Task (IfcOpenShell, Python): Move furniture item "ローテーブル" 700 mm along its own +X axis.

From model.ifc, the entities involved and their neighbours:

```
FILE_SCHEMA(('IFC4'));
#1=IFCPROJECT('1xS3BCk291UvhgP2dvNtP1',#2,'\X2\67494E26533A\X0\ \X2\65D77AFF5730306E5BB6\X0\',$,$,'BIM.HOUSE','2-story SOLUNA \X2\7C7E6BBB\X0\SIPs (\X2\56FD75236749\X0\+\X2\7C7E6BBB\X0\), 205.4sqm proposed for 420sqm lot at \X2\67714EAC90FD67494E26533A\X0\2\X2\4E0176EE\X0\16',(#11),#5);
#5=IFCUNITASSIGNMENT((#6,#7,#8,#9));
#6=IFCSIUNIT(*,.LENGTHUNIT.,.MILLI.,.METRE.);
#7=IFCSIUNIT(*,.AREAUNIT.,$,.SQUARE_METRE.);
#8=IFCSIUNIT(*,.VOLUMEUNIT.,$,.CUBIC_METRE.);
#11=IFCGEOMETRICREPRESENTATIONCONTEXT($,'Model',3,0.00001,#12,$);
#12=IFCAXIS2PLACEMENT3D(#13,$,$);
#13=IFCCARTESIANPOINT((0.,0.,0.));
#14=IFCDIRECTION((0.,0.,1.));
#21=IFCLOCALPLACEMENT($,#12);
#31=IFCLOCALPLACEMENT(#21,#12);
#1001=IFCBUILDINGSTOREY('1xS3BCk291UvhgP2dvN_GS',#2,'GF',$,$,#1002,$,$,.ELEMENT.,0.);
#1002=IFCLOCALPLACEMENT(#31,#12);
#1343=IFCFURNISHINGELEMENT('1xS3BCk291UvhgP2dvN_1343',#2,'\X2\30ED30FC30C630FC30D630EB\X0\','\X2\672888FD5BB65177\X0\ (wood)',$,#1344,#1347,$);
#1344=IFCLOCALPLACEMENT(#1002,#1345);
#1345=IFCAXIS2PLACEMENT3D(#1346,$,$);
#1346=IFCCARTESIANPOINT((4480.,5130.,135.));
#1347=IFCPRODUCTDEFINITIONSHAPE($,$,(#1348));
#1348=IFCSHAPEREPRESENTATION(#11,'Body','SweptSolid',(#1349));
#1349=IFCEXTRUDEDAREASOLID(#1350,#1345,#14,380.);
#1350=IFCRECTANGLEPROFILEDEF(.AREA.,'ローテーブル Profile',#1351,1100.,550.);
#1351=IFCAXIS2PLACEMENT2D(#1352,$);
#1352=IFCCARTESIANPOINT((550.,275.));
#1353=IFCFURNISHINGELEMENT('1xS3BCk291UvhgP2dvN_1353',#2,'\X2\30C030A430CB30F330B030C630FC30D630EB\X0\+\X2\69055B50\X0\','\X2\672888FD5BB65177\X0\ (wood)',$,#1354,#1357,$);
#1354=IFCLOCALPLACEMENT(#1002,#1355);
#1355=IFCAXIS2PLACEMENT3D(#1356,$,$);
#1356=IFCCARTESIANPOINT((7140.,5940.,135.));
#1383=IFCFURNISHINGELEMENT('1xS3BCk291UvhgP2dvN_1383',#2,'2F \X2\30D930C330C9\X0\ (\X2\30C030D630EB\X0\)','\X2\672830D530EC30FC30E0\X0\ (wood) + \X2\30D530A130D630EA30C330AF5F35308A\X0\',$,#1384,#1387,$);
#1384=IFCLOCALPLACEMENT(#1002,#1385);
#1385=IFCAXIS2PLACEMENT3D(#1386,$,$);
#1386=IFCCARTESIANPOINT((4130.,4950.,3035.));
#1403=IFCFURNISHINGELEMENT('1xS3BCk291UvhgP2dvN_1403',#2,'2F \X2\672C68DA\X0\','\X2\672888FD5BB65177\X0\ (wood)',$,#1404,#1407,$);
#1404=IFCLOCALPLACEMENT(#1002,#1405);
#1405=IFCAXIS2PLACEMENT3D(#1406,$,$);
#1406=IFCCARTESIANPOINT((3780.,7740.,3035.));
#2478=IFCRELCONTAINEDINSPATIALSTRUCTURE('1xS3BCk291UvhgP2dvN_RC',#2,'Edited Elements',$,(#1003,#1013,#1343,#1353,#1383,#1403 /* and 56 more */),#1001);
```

```python
import ifcopenshell
import ifcopenshell.api.geometry
import ifcopenshell.util.placement

model = ifcopenshell.open("model.ifc")

item = model.by_id(1343)
matrix = ifcopenshell.util.placement.get_local_placement(item.ObjectPlacement)
matrix[:3, 3] += matrix[:3, 0] * 700.0
ifcopenshell.api.geometry.edit_object_placement(model, product=item, matrix=matrix, is_si=False)

print(ifcopenshell.util.placement.get_local_placement(item.ObjectPlacement).round(3) + 0.0)

model.write("model_v2.ifc")
```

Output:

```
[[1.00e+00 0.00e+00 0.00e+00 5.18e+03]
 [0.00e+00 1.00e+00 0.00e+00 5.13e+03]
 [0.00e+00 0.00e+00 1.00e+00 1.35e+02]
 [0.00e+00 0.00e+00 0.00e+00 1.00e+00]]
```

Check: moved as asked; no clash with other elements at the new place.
